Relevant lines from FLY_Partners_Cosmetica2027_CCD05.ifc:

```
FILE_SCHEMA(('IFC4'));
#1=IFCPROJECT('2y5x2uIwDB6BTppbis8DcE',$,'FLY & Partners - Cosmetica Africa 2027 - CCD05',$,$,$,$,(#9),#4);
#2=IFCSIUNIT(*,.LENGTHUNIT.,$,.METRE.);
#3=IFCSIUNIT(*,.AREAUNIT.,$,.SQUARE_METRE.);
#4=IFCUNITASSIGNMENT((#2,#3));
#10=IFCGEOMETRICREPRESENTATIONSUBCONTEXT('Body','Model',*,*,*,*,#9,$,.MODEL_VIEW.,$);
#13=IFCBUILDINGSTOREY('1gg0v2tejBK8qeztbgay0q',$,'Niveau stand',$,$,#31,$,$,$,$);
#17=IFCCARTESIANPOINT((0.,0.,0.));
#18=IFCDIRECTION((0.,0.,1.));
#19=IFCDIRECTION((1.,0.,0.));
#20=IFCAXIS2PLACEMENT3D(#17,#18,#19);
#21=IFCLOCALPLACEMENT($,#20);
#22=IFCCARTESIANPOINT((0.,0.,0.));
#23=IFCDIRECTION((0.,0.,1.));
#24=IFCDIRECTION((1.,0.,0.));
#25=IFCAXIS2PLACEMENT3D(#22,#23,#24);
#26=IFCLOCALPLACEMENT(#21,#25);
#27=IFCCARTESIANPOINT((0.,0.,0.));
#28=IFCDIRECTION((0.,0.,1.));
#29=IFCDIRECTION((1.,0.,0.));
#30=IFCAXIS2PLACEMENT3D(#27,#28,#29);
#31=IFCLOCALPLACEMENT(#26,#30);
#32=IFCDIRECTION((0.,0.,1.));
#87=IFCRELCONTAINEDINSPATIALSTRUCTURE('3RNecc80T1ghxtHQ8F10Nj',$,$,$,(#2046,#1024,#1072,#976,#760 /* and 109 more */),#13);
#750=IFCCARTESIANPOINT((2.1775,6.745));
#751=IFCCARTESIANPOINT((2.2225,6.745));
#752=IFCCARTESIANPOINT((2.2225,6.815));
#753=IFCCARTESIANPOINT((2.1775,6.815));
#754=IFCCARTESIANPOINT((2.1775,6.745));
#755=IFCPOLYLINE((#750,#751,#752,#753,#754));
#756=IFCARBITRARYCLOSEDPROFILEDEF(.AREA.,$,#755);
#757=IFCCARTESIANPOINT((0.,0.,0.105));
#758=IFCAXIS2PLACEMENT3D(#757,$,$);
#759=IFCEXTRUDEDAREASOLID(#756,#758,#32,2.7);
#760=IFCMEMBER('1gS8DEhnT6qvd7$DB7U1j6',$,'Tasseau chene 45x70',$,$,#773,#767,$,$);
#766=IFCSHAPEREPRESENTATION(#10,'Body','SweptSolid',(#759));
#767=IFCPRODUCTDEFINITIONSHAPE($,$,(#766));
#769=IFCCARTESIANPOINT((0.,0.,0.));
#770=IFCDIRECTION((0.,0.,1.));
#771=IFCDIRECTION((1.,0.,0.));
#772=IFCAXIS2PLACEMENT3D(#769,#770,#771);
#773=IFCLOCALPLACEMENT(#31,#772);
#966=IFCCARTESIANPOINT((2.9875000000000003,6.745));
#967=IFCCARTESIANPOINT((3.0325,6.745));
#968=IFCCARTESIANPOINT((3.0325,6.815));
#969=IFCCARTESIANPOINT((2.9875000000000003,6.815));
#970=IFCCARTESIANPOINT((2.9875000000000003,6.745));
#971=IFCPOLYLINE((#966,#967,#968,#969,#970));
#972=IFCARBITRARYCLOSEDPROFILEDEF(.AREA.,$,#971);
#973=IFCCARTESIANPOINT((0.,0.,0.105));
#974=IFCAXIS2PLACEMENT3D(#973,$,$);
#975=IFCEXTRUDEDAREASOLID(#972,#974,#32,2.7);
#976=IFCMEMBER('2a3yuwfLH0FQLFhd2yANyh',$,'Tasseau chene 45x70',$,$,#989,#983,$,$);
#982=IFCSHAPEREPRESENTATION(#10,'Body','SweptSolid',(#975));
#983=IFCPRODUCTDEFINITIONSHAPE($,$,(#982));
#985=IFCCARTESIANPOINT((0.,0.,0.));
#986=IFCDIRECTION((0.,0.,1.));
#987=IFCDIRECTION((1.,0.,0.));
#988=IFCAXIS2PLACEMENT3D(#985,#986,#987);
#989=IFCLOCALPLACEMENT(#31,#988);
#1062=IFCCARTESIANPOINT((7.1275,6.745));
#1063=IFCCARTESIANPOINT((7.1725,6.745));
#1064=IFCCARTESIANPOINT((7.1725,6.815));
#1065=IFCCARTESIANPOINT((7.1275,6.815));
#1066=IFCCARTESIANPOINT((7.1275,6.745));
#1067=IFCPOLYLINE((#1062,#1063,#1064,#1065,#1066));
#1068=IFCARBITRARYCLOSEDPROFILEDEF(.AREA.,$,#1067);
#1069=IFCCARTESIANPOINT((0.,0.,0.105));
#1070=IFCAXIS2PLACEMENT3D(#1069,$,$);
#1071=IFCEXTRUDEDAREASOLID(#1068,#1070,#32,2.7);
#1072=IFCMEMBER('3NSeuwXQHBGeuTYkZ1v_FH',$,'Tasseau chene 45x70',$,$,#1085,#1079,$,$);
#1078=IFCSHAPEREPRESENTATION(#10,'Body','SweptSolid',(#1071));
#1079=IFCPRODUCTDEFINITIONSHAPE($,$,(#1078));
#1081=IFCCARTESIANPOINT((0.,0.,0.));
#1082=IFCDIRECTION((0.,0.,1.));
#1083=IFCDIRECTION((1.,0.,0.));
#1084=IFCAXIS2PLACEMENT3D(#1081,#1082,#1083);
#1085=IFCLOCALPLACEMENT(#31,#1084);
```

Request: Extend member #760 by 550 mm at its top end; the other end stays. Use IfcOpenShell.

```python
import ifcopenshell
import ifcopenshell.util.representation

model = ifcopenshell.open("FLY_Partners_Cosmetica2027_CCD05.ifc")

member = model.by_id(760)
change = 0.55

# The extrusion runs towards the end named, so only its depth changes.
body = ifcopenshell.util.representation.get_representation(member, "Model", "Body")
solid = body.Items[0]
old_length = solid.Depth
solid.Depth += change

print(f"length {old_length:g} -> {solid.Depth:g}")

model.write("FLY_Partners_Cosmetica2027_CCD05-out.ifc")
```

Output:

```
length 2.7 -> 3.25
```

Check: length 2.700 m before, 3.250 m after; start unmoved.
